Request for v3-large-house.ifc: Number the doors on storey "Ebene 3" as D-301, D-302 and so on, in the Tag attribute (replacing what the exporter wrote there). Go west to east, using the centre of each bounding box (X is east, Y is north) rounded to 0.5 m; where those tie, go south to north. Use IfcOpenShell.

First a look at what the model holds.

```python
import ifcopenshell
import ifcopenshell.util.element
import ifcopenshell.util.placement

model = ifcopenshell.open("v3-large-house.ifc")
print(model.schema)
storey = next(s for s in model.by_type("IfcBuildingStorey") if s.Name == "Ebene 3")
doors = [e for e in ifcopenshell.util.element.get_decomposition(storey) if e.is_a("IfcDoor")]
for e in sorted(doors, key=lambda e: e.id()):
    origin = ifcopenshell.util.placement.get_local_placement(e.ObjectPlacement)[:3, 3]
    print(e.id(), e.Tag, e.Name, origin.round(2) + 0.0, sep=" | ")
```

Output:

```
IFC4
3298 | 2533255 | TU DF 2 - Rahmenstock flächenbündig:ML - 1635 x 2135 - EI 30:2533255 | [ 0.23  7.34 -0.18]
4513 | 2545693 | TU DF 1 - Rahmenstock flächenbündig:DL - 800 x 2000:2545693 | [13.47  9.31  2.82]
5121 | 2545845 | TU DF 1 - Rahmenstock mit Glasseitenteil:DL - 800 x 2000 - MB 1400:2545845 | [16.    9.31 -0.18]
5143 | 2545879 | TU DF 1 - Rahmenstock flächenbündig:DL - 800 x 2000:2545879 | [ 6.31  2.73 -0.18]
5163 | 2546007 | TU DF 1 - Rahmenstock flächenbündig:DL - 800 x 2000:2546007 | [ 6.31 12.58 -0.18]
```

```python
import ifcopenshell
import ifcopenshell.geom
import ifcopenshell.util.element
import ifcopenshell.util.shape

model = ifcopenshell.open("v3-large-house.ifc")
settings = ifcopenshell.geom.settings()
settings.set("use-world-coords", True)


def centre(element):
    shape = ifcopenshell.geom.create_shape(settings, element)
    return ifcopenshell.util.shape.get_bbox_centroid(shape.geometry)


storey = next(s for s in model.by_type("IfcBuildingStorey") if s.Name == "Ebene 3")
doors = [e for e in ifcopenshell.util.element.get_decomposition(storey) if e.is_a("IfcDoor")]

# Insertion points can sit at a corner or the storey origin, so sort by the geometry (in metres).
centres = {e: centre(e) for e in doors}
doors.sort(key=lambda e: (round(centres[e][0] / 0.5), centres[e][1]))

for i, e in enumerate(doors, start=1):
    number = f"D-3{i:02d}"
    e.Tag = number
    print(e.id(), number)

model.write("v3-large-house_rev.ifc")
```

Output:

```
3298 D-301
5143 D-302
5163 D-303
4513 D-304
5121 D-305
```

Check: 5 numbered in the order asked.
